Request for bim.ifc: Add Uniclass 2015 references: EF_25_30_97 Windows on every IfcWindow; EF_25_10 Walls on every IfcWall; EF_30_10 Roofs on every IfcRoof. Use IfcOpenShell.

First a look at what the model holds.

```python
import ifcopenshell

model = ifcopenshell.open("bim.ifc")
print(model.schema)
print("classifications:", [c.Name for c in model.by_type("IfcClassification")])
for ifc_class in ("IfcDoor", "IfcRoof", "IfcStair", "IfcWall", "IfcWindow"):
    print(ifc_class, len(model.by_type(ifc_class)))
```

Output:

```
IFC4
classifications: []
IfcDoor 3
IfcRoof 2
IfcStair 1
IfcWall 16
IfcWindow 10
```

```python
import ifcopenshell
import ifcopenshell.api.classification

model = ifcopenshell.open("bim.ifc")

system = ifcopenshell.api.classification.add_classification(model, classification="Uniclass 2015")

codes = {
    "IfcWindow": ("EF_25_30_97", "Windows"),
    "IfcWall": ("EF_25_10", "Walls"),
    "IfcRoof": ("EF_30_10", "Roofs"),
}
for ifc_class, (code, name) in codes.items():
    products = model.by_type(ifc_class)
    ifcopenshell.api.classification.add_reference(
        model, products=products, classification=system, identification=code, name=name
    )
    print(code, len(products))

model.write("bim_updated.ifc")
```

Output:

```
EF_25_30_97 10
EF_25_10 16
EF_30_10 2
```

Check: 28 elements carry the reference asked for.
